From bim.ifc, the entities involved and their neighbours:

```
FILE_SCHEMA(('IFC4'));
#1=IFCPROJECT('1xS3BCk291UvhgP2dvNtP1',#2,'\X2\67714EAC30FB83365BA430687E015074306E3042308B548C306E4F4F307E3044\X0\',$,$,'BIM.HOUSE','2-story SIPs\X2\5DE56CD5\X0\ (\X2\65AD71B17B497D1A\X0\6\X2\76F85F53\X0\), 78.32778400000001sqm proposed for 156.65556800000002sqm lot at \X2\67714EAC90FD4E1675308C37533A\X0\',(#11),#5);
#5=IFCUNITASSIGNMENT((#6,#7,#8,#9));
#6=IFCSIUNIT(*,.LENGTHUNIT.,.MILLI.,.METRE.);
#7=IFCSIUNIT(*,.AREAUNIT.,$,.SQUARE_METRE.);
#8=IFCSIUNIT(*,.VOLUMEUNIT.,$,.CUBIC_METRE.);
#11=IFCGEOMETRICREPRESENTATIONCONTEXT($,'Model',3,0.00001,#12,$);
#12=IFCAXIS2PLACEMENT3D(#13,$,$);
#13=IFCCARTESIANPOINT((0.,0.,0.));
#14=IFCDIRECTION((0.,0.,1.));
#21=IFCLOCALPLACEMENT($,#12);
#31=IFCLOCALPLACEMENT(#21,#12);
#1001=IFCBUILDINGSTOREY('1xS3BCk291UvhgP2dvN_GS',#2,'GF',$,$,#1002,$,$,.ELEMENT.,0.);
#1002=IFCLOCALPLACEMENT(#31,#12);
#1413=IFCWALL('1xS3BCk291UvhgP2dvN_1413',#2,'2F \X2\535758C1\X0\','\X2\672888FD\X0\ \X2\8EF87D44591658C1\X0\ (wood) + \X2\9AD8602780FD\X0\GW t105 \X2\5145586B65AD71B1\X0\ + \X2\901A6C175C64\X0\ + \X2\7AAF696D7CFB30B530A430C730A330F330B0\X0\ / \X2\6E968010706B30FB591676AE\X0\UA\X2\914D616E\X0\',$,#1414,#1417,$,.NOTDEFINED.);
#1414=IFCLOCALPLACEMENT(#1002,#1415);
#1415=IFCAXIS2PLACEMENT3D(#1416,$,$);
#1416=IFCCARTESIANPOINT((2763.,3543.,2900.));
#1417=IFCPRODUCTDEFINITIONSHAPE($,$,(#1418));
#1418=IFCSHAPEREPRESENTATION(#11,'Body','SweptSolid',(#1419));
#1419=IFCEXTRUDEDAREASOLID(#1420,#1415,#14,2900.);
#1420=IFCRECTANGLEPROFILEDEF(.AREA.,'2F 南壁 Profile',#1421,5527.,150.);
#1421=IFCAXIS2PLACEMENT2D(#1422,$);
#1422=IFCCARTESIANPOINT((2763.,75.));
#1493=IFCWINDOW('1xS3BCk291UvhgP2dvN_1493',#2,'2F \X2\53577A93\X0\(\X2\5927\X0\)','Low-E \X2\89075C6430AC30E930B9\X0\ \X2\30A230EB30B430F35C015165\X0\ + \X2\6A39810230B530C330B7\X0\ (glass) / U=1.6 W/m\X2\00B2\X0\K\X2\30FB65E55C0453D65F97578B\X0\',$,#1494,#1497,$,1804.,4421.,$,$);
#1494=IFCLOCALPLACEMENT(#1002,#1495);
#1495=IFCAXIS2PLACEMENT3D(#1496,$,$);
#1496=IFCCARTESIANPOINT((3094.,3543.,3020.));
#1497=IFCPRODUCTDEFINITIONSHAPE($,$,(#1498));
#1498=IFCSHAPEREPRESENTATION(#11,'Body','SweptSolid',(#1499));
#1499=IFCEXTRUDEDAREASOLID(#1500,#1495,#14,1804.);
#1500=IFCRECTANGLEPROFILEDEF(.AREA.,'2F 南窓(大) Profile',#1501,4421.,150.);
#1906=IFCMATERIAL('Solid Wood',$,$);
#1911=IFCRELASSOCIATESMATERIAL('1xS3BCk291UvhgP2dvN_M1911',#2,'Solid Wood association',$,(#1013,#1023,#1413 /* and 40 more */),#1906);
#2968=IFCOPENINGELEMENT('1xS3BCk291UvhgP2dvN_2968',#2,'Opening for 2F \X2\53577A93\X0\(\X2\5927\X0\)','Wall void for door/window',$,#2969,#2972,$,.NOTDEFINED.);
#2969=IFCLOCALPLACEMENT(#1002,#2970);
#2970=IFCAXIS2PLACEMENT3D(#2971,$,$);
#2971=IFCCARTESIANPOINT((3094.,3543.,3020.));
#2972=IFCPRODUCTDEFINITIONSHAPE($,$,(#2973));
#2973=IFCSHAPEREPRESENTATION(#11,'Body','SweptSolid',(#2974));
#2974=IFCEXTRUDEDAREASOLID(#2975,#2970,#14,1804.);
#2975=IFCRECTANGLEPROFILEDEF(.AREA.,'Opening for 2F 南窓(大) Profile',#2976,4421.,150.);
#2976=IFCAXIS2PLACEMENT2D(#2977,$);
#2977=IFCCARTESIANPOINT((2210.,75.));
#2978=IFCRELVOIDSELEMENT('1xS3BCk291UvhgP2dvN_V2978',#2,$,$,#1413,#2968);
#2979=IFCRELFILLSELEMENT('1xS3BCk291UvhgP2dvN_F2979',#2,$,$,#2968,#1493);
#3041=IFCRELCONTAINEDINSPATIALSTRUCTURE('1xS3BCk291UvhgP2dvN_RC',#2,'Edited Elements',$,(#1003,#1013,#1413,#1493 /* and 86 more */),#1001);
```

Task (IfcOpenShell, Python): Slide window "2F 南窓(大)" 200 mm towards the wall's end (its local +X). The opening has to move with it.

```python
import ifcopenshell
import ifcopenshell.api.geometry
import ifcopenshell.util.placement

model = ifcopenshell.open("bim.ifc")

window = model.by_guid("1xS3BCk291UvhgP2dvN_1493")
opening = window.FillsVoids[0].RelatingOpeningElement
wall = opening.VoidsElements[0].RelatingBuildingElement

wall_matrix = ifcopenshell.util.placement.get_local_placement(wall.ObjectPlacement)
shift = wall_matrix[:3, 0] * 200.0
before = ifcopenshell.util.placement.get_local_placement(window.ObjectPlacement)[:3, 3].copy()

# The window is not placed relative to its opening, so move both.
for product in (opening, window):
    matrix = ifcopenshell.util.placement.get_local_placement(product.ObjectPlacement)
    matrix[:3, 3] += shift
    ifcopenshell.api.geometry.edit_object_placement(model, product=product, matrix=matrix, is_si=False)

after = ifcopenshell.util.placement.get_local_placement(window.ObjectPlacement)[:3, 3]
print("window moved by", (after - before).round(3) + 0.0)

model.write("bim_edited.ifc")
```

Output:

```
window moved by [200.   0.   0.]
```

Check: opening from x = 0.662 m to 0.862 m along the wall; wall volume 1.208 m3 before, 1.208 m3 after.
